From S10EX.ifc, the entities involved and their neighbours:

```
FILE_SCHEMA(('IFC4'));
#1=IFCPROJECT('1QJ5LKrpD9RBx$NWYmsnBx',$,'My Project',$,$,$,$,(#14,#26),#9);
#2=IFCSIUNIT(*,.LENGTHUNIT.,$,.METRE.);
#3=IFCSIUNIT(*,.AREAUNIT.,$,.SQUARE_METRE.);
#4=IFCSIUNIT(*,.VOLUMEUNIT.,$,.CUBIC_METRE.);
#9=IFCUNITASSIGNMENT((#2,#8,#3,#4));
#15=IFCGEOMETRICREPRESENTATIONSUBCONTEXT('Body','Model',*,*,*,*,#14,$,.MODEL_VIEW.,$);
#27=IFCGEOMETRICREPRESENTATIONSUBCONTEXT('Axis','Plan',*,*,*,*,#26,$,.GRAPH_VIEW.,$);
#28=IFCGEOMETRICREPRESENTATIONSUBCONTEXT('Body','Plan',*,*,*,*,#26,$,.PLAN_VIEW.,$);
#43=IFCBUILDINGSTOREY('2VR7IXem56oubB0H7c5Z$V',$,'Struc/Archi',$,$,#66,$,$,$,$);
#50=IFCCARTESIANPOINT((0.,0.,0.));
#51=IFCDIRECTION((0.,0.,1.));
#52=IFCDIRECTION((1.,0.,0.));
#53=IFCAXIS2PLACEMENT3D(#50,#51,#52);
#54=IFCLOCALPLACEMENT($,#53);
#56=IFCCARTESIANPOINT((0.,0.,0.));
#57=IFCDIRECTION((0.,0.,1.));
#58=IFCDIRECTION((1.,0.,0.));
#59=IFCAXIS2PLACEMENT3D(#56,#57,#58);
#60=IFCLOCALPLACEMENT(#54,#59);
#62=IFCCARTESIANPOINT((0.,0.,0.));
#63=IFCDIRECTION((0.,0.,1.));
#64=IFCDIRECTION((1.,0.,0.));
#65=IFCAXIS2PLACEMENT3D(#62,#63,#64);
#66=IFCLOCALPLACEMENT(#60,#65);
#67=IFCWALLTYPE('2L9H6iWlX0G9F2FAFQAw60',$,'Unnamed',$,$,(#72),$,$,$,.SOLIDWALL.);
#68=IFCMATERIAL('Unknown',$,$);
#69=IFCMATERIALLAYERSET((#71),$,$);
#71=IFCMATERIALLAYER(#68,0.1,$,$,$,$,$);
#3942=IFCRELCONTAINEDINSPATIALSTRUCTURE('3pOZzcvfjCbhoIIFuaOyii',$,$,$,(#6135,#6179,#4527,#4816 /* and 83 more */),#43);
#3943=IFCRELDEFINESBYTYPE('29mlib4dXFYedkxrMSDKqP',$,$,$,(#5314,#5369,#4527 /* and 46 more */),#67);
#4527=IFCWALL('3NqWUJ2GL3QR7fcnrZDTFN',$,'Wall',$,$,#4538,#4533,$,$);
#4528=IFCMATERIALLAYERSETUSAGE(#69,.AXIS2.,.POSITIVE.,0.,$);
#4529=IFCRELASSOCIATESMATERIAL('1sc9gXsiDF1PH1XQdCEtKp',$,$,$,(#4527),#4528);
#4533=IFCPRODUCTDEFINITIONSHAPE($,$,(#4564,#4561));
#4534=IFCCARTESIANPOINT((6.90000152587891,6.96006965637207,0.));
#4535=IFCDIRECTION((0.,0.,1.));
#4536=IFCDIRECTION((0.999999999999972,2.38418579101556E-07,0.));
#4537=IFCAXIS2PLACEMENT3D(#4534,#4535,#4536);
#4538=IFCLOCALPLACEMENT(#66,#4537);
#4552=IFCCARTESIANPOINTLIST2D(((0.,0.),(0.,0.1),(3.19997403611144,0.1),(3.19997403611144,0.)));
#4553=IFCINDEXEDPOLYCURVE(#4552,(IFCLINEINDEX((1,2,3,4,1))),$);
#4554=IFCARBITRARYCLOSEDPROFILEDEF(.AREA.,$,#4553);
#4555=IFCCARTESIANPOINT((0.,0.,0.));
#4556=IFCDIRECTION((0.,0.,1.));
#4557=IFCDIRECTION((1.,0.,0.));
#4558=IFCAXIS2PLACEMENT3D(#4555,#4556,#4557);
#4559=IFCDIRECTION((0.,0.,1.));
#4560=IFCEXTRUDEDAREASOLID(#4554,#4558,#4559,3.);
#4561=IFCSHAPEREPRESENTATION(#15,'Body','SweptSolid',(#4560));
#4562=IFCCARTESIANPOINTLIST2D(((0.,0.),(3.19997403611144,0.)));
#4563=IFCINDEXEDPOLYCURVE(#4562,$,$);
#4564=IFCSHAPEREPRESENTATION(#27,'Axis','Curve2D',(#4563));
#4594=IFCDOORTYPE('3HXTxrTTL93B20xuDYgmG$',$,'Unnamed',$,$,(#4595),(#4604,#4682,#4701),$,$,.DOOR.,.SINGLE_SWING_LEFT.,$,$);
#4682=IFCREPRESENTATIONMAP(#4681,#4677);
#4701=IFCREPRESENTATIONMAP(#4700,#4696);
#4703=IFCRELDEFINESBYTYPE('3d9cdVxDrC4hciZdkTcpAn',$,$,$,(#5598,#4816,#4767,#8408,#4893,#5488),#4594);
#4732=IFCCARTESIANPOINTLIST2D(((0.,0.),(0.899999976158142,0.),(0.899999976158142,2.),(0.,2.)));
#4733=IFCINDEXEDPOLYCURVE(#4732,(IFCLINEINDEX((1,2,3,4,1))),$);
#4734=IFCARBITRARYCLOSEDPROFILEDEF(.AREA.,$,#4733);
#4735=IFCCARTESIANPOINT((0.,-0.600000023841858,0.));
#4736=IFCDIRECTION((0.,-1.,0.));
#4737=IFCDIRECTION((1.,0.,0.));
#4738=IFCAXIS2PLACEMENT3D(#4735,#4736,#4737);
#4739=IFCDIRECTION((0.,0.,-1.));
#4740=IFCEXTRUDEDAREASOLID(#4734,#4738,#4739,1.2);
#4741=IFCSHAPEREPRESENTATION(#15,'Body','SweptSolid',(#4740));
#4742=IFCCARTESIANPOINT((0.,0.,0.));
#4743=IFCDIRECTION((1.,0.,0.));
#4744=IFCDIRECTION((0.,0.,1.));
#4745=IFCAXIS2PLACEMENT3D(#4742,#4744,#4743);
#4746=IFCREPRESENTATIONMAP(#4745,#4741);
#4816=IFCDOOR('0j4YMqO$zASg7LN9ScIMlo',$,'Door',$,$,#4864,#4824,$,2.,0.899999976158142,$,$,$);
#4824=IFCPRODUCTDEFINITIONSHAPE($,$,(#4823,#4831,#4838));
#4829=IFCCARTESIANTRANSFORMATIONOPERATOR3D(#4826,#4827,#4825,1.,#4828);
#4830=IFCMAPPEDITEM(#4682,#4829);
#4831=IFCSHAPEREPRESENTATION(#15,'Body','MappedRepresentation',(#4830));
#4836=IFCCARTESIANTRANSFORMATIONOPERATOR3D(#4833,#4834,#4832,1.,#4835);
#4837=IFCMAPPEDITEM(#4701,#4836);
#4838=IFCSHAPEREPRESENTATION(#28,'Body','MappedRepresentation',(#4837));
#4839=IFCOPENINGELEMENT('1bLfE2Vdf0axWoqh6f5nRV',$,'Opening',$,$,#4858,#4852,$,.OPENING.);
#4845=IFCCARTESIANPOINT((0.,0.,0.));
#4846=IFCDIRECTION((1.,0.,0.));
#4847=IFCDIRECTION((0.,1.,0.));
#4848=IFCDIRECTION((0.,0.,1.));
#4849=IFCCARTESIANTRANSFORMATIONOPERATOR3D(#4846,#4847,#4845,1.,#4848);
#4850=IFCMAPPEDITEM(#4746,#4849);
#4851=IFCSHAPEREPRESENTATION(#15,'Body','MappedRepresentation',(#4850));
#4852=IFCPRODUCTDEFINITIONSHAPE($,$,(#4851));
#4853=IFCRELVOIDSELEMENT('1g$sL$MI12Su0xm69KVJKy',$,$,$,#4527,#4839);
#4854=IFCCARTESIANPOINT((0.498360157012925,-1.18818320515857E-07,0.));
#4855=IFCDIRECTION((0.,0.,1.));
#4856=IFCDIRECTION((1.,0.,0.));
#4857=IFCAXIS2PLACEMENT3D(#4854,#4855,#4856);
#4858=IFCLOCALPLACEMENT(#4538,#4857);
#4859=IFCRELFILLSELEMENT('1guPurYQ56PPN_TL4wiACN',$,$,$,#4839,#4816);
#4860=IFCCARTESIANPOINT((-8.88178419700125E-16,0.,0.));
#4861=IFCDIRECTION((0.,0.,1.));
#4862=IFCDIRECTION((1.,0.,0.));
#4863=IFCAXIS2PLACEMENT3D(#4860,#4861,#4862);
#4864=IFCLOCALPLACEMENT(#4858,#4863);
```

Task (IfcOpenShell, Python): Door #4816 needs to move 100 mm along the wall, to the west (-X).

```python
import ifcopenshell
import ifcopenshell.api.geometry
import ifcopenshell.util.placement
import ifcopenshell.util.unit

model = ifcopenshell.open("S10EX.ifc")
unit_scale = ifcopenshell.util.unit.calculate_unit_scale(model)

door = model.by_id(4816)
opening = door.FillsVoids[0].RelatingOpeningElement
wall = opening.VoidsElements[0].RelatingBuildingElement

wall_matrix = ifcopenshell.util.placement.get_local_placement(wall.ObjectPlacement)
shift = wall_matrix[:3, 0] * -0.1 / unit_scale
before = ifcopenshell.util.placement.get_local_placement(door.ObjectPlacement)[:3, 3].copy()

# The door is placed relative to its opening, so it follows when the opening moves.
matrix = ifcopenshell.util.placement.get_local_placement(opening.ObjectPlacement)
matrix[:3, 3] += shift
ifcopenshell.api.geometry.edit_object_placement(
    model, product=opening, matrix=matrix, is_si=False, should_transform_children=True
)

after = ifcopenshell.util.placement.get_local_placement(door.ObjectPlacement)[:3, 3]
print("door moved by", (after - before).round(3) + 0.0)

model.write("S10EX_updated.ifc")
```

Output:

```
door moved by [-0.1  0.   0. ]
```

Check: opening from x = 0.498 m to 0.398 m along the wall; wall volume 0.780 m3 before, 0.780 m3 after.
